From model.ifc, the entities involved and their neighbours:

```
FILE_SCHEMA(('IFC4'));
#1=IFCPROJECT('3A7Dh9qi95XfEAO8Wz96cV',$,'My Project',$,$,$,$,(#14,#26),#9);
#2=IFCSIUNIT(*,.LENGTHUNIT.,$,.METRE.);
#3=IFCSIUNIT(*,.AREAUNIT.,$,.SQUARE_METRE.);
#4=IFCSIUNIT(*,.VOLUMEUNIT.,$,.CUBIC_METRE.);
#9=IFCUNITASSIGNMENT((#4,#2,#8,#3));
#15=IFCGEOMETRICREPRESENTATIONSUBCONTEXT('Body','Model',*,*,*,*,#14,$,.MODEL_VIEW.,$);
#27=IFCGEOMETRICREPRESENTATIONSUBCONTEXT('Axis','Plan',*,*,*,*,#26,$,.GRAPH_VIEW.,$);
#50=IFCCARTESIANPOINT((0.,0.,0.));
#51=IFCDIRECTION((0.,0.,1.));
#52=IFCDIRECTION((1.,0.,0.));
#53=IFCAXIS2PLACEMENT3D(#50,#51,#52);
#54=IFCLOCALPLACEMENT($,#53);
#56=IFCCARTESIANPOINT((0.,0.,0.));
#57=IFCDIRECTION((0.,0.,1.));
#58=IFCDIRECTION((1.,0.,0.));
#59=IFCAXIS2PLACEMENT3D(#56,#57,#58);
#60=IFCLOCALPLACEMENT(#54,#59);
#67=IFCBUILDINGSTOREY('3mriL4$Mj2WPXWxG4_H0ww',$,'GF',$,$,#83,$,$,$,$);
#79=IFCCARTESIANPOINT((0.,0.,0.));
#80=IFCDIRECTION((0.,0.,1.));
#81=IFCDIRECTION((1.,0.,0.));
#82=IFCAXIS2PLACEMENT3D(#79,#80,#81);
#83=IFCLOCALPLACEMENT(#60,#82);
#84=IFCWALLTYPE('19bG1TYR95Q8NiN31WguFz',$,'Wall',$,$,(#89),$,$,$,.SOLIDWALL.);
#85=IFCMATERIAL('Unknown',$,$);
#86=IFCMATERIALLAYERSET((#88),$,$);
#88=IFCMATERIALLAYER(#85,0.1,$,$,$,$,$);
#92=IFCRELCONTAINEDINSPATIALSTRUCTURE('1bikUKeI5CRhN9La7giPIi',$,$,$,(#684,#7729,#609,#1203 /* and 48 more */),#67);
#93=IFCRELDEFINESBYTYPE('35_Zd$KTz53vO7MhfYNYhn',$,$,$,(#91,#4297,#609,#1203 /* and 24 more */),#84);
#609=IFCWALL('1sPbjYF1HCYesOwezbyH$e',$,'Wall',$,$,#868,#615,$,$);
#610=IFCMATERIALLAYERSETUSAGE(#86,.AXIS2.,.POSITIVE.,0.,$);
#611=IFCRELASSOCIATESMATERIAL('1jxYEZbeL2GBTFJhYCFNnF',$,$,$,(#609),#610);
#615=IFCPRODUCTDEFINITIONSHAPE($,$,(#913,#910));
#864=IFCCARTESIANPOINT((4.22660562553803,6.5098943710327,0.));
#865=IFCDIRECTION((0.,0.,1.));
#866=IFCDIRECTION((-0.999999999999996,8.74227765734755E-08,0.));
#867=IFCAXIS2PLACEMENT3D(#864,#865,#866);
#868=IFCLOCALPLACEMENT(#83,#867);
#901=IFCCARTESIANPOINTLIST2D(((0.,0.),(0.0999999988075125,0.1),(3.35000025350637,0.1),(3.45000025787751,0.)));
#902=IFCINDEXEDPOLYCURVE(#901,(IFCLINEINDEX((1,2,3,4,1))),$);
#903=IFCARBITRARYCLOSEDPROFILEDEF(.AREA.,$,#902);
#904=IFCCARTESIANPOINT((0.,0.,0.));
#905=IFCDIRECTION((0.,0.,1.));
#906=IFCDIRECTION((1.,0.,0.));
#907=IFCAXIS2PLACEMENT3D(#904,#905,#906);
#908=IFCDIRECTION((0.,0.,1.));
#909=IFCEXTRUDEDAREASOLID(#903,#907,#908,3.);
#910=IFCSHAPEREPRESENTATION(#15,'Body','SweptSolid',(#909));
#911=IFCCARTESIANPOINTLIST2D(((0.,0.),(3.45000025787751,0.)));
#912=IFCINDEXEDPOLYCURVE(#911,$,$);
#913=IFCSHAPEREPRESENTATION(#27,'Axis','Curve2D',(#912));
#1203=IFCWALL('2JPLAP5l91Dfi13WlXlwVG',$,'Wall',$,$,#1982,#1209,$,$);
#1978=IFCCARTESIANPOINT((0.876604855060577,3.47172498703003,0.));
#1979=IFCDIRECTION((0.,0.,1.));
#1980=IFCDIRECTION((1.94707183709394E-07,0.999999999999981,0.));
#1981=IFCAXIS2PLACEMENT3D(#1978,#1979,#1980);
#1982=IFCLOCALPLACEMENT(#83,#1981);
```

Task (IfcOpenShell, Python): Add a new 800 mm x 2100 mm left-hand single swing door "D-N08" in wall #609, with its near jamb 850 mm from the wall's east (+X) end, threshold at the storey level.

```python
import numpy as np
import ifcopenshell
import ifcopenshell.api.feature
import ifcopenshell.api.geometry
import ifcopenshell.api.root
import ifcopenshell.api.spatial
import ifcopenshell.geom
import ifcopenshell.util.element
import ifcopenshell.util.placement
import ifcopenshell.util.representation
import ifcopenshell.util.shape
import ifcopenshell.util.unit

model = ifcopenshell.open("model.ifc")
unit_scale = ifcopenshell.util.unit.calculate_unit_scale(model)
settings = ifcopenshell.geom.settings()


def volume(element):
    """Net volume in cubic metres, openings subtracted."""
    shape = ifcopenshell.geom.create_shape(settings, element)
    return ifcopenshell.util.shape.get_volume(shape.geometry)


wall = model.by_guid("1sPbjYF1HCYesOwezbyH$e")
storey = ifcopenshell.util.element.get_container(wall, ifc_class="IfcBuildingStorey")
context = ifcopenshell.util.representation.get_context(model, "Model", "Body", "MODEL_VIEW")
before = volume(wall)

width, height, from_end, sill = 0.8, 2.1, 0.85, 0.0  # metres

# The wall runs along its own X axis, and the end named is its -X end.
wall_shape = ifcopenshell.geom.create_shape(settings, wall)
x, y, z = ifcopenshell.util.shape.get_vertices(wall_shape.geometry).T
start = x.min() + from_end
face, thickness = float(y.min()), float(y.max() - y.min())
wall_matrix = ifcopenshell.util.placement.get_local_placement(wall.ObjectPlacement)
level = ifcopenshell.util.placement.get_local_placement(storey.ObjectPlacement)[2, 3]


def in_wall(x, y):
    """Placement at x, y metres in the wall's axes, at sill height."""
    matrix = wall_matrix.copy()
    matrix[:, 3] = wall_matrix @ np.array([x / unit_scale, y / unit_scale, 0.0, 1.0])
    matrix[2, 3] = level + sill / unit_scale
    return matrix


# Opening: a box that overshoots both wall faces by 50 mm.
opening = ifcopenshell.api.root.create_entity(model, ifc_class="IfcOpeningElement", predefined_type="OPENING")
box = ifcopenshell.api.geometry.add_wall_representation(
    model, context=context, length=width, height=height, thickness=thickness + 0.1
)
ifcopenshell.api.geometry.assign_representation(model, product=opening, representation=box)
ifcopenshell.api.geometry.edit_object_placement(model, product=opening, matrix=in_wall(start, face - 0.05), is_si=False)
ifcopenshell.api.feature.add_feature(model, feature=opening, element=wall)

door = ifcopenshell.api.root.create_entity(model, ifc_class="IfcDoor", name="D-N08", predefined_type="DOOR")
door.OverallWidth, door.OverallHeight = width / unit_scale, height / unit_scale
door.OperationType = "SINGLE_SWING_LEFT"
body = ifcopenshell.api.geometry.add_door_representation(
    model,
    context=context,
    overall_width=door.OverallWidth,
    overall_height=door.OverallHeight,
    operation_type="SINGLE_SWING_LEFT",
    lining_properties={"LiningDepth": thickness / unit_scale, "ThresholdDepth": thickness / unit_scale},
)
ifcopenshell.api.geometry.assign_representation(model, product=door, representation=body)
ifcopenshell.api.spatial.assign_container(model, products=[door], relating_structure=storey)
ifcopenshell.api.feature.add_filling(model, opening=opening, element=door)

# The lining spans the wall, so the door starts at the wall face.
ifcopenshell.api.geometry.edit_object_placement(model, product=door, matrix=in_wall(start, face), is_si=False)

after = volume(wall)

print(f"wall volume {before:.3f} -> {after:.3f} m3")

model.write("model_updated.ifc")
```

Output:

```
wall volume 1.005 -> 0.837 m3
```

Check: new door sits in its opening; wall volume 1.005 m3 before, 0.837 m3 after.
